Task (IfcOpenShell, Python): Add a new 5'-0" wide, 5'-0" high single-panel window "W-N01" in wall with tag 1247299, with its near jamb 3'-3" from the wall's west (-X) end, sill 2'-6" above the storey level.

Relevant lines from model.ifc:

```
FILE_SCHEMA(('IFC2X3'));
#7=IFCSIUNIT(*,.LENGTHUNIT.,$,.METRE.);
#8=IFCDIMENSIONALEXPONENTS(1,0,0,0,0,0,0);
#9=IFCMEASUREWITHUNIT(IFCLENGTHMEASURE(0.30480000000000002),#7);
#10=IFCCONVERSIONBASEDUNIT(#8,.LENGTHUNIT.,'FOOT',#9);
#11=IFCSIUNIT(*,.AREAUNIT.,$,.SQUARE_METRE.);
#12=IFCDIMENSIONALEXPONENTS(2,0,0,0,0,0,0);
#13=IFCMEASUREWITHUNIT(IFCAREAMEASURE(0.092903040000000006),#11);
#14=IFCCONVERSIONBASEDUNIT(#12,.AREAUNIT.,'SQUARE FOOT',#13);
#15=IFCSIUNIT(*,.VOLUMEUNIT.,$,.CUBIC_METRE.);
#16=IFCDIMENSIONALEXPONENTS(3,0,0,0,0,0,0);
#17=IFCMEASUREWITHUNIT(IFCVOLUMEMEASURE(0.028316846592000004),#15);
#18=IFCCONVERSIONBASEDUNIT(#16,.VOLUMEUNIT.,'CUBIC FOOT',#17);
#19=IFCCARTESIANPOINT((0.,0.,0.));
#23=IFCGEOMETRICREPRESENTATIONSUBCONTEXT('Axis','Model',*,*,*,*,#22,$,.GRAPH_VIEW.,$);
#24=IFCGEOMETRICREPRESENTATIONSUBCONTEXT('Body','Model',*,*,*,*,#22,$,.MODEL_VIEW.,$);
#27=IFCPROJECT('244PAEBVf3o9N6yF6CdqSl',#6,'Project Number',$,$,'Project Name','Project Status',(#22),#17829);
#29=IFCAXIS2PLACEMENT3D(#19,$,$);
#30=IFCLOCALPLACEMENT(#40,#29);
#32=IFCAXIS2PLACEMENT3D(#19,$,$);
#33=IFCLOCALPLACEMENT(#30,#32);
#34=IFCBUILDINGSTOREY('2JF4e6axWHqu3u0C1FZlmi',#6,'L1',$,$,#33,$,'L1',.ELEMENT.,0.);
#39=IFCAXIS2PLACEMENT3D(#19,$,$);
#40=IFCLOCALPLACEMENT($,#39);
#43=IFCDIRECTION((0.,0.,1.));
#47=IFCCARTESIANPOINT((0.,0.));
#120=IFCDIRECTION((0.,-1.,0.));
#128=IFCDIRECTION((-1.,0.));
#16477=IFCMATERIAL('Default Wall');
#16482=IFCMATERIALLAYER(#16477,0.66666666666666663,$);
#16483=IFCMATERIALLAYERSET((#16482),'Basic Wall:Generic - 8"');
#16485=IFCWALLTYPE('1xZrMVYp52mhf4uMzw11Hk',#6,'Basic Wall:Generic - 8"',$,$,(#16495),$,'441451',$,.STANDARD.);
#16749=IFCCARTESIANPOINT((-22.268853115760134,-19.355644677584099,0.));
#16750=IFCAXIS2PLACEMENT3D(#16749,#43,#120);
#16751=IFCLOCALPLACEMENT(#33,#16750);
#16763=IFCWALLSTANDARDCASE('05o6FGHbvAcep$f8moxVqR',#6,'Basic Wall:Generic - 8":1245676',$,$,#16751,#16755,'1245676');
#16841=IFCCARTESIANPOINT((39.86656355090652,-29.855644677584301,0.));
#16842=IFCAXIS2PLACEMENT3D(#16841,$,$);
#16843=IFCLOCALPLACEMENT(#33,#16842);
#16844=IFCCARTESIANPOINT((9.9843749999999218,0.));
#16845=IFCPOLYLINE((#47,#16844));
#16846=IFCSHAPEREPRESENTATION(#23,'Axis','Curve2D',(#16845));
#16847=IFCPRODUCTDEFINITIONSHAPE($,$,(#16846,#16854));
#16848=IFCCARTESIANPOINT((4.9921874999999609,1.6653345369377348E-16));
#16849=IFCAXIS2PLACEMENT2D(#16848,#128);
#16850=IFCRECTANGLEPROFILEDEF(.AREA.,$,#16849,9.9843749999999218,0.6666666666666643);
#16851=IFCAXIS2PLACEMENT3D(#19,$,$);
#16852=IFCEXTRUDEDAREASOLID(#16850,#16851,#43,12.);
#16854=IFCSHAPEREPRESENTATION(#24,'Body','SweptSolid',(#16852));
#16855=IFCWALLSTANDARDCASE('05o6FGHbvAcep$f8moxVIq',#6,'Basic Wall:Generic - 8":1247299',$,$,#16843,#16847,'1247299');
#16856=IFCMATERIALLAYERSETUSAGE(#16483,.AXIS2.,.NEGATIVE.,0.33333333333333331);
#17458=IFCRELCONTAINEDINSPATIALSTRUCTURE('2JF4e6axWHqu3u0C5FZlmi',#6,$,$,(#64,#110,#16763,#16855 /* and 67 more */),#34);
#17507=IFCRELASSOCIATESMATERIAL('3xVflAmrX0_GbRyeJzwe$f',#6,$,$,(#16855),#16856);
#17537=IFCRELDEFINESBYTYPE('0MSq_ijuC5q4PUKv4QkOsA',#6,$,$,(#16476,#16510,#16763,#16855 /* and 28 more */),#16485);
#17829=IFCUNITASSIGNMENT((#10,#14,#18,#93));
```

```python
import numpy as np
import ifcopenshell
import ifcopenshell.api.feature
import ifcopenshell.api.geometry
import ifcopenshell.api.root
import ifcopenshell.api.spatial
import ifcopenshell.api.type
import ifcopenshell.geom
import ifcopenshell.util.element
import ifcopenshell.util.placement
import ifcopenshell.util.representation
import ifcopenshell.util.shape
import ifcopenshell.util.unit

model = ifcopenshell.open("model.ifc")
unit_scale = ifcopenshell.util.unit.calculate_unit_scale(model)
settings = ifcopenshell.geom.settings()


def volume(element):
    """Net volume in cubic metres, openings subtracted."""
    shape = ifcopenshell.geom.create_shape(settings, element)
    return ifcopenshell.util.shape.get_volume(shape.geometry)


wall = model.by_guid("05o6FGHbvAcep$f8moxVIq")
storey = ifcopenshell.util.element.get_container(wall, ifc_class="IfcBuildingStorey")
context = ifcopenshell.util.representation.get_context(model, "Model", "Body", "MODEL_VIEW")
before = volume(wall)

width, height, from_end, sill = 1.524, 1.524, 0.9906, 0.762  # metres

# The wall runs along its own X axis, and the end named is its -X end.
wall_shape = ifcopenshell.geom.create_shape(settings, wall)
x, y, z = ifcopenshell.util.shape.get_vertices(wall_shape.geometry).T
start = x.min() + from_end
face, thickness = float(y.min()), float(y.max() - y.min())
wall_matrix = ifcopenshell.util.placement.get_local_placement(wall.ObjectPlacement)
level = ifcopenshell.util.placement.get_local_placement(storey.ObjectPlacement)[2, 3]


def in_wall(x, y):
    """Placement at x, y metres in the wall's axes, at sill height."""
    matrix = wall_matrix.copy()
    matrix[:, 3] = wall_matrix @ np.array([x / unit_scale, y / unit_scale, 0.0, 1.0])
    matrix[2, 3] = level + sill / unit_scale
    return matrix


# Opening: a box that overshoots both wall faces by 50 mm.
opening = ifcopenshell.api.root.create_entity(model, ifc_class="IfcOpeningElement")
box = ifcopenshell.api.geometry.add_wall_representation(
    model, context=context, length=width, height=height, thickness=thickness + 0.1
)
ifcopenshell.api.geometry.assign_representation(model, product=opening, representation=box)
ifcopenshell.api.geometry.edit_object_placement(model, product=opening, matrix=in_wall(start, face - 0.05), is_si=False)
ifcopenshell.api.feature.add_feature(model, feature=opening, element=wall)

window = ifcopenshell.api.root.create_entity(model, ifc_class="IfcWindow", name="W-N01")
window.OverallWidth, window.OverallHeight = width / unit_scale, height / unit_scale
body = ifcopenshell.api.geometry.add_window_representation(
    model,
    context=context,
    overall_width=window.OverallWidth,
    overall_height=window.OverallHeight,
    partition_type="SINGLE_PANEL",
)
ifcopenshell.api.geometry.assign_representation(model, product=window, representation=body)
ifcopenshell.api.spatial.assign_container(model, products=[window], relating_structure=storey)
fills = ifcopenshell.api.feature.add_filling(model, opening=opening, element=window)
fills.OwnerHistory = window.OwnerHistory  # required in IFC2X3

# IFC2X3 keeps the operation on the window style.
style = ifcopenshell.api.root.create_entity(model, ifc_class="IfcWindowStyle", name="W-N01")
style.OperationType, style.ConstructionType = "SINGLE_PANEL", "NOTDEFINED"
style.ParameterTakesPrecedence = style.Sizeable = False
ifcopenshell.api.type.assign_type(model, related_objects=[window], relating_type=style)

# Centre the window in the wall's thickness.
ifcopenshell.api.geometry.edit_object_placement(model, product=window, matrix=in_wall(start, face), is_si=False)
window_shape = ifcopenshell.geom.create_shape(settings, window)
depth = ifcopenshell.util.shape.get_vertices(window_shape.geometry)[:, 1]
offset = face + thickness / 2 - (depth.min() + depth.max()) / 2
ifcopenshell.api.geometry.edit_object_placement(model, product=window, matrix=in_wall(start, offset), is_si=False)

after = volume(wall)

print(f"wall volume {before:.3f} -> {after:.3f} m3")

model.write("model_v2.ifc")
```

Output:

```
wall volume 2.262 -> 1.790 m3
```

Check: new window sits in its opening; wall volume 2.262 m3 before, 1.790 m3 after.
